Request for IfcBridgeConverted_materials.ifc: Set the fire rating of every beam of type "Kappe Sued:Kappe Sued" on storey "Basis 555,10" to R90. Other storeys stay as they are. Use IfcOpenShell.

First a look at what the model holds.

```python
import ifcopenshell
import ifcopenshell.util.element

model = ifcopenshell.open("IfcBridgeConverted_materials.ifc")
print(model.schema)
storey = next(s for s in model.by_type("IfcBuildingStorey") if s.Name == "Basis 555,10")
beams = [e for e in ifcopenshell.util.element.get_decomposition(storey) if e.is_a("IfcBeam")]
seen = {}
for e in beams:
    element_type = ifcopenshell.util.element.get_type(e)
    key = (element_type.Name if element_type != e and element_type else None, ifcopenshell.util.element.get_pset(e, "Pset_BeamCommon", "FireRating"))
    seen[key] = seen.get(key, 0) + 1
for (name, value), count in sorted(seen.items(), key=str):
    print(count, "x", name, "|", value)
```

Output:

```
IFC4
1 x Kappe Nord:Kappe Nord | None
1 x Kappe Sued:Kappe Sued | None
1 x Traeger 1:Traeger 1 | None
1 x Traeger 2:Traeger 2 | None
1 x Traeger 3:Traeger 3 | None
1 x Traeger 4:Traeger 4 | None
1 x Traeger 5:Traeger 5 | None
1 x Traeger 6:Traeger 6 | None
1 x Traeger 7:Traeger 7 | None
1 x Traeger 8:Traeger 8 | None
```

```python
import ifcopenshell
import ifcopenshell.api.pset
import ifcopenshell.util.element

model = ifcopenshell.open("IfcBridgeConverted_materials.ifc")

storey = next(s for s in model.by_type("IfcBuildingStorey") if s.Name == "Basis 555,10")
beams = [e for e in ifcopenshell.util.element.get_decomposition(storey) if e.is_a("IfcBeam")]

count = 0
for e in beams:
    element_type = ifcopenshell.util.element.get_type(e)
    if element_type in (None, e) or element_type.Name != "Kappe Sued:Kappe Sued":
        continue
    # add_pset returns the element's existing set when there is one.
    pset = ifcopenshell.api.pset.add_pset(model, product=e, name="Pset_BeamCommon")
    ifcopenshell.api.pset.edit_pset(model, pset=pset, properties={"FireRating": "R90"})
    count += 1

print(count, "beams updated")

model.write("IfcBridgeConverted_materials_v2.ifc")
```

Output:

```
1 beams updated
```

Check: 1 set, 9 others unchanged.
